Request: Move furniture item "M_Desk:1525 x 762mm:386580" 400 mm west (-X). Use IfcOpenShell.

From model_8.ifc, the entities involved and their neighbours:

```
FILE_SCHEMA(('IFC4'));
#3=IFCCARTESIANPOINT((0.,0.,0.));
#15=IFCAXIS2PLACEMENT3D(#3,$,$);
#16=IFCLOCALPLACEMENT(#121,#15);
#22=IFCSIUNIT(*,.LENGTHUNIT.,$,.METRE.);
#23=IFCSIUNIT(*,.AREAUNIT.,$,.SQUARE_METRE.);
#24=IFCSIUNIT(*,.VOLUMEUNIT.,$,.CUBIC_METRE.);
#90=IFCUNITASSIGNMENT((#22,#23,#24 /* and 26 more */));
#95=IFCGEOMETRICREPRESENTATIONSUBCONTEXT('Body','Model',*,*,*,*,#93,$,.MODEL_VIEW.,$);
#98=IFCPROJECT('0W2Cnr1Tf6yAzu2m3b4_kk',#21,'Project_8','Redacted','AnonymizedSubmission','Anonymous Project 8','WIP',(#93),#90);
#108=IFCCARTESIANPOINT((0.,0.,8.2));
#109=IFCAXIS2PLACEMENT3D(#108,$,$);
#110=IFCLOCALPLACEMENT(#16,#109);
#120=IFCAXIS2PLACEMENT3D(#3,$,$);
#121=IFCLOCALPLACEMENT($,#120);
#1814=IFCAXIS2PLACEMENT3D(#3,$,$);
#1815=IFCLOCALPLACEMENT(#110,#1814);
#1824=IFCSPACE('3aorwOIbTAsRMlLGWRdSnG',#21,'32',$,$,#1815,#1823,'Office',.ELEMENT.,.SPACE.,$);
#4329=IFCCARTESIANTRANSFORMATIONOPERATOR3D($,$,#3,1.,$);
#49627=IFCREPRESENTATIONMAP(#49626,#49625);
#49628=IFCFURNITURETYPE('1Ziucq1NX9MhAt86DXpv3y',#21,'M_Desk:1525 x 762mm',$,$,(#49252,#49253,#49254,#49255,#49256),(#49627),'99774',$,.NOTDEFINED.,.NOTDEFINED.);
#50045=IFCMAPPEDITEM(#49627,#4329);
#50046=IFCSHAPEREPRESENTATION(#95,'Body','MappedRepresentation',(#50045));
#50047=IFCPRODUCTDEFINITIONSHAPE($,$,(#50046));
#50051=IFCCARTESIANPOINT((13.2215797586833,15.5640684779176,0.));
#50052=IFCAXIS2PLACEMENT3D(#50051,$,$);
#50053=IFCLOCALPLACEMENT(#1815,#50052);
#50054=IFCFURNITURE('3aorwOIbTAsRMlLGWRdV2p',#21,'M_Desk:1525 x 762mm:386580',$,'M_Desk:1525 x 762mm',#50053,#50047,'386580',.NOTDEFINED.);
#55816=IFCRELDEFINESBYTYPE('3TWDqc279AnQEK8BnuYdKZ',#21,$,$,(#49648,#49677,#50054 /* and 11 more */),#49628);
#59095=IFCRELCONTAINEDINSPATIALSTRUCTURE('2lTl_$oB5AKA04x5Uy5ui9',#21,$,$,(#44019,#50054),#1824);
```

```python
import ifcopenshell
import ifcopenshell.api.geometry
import ifcopenshell.util.placement
import ifcopenshell.util.unit

model = ifcopenshell.open("model_8.ifc")
unit_scale = ifcopenshell.util.unit.calculate_unit_scale(model)

item = model.by_id(50054)
matrix = ifcopenshell.util.placement.get_local_placement(item.ObjectPlacement)
matrix[0, 3] -= 0.4 / unit_scale
ifcopenshell.api.geometry.edit_object_placement(model, product=item, matrix=matrix, is_si=False)

print(ifcopenshell.util.placement.get_local_placement(item.ObjectPlacement).round(3) + 0.0)

model.write("model_8_edited.ifc")
```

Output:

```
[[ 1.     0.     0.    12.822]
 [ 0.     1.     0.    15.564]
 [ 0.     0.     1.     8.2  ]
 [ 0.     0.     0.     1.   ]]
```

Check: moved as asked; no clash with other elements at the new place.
